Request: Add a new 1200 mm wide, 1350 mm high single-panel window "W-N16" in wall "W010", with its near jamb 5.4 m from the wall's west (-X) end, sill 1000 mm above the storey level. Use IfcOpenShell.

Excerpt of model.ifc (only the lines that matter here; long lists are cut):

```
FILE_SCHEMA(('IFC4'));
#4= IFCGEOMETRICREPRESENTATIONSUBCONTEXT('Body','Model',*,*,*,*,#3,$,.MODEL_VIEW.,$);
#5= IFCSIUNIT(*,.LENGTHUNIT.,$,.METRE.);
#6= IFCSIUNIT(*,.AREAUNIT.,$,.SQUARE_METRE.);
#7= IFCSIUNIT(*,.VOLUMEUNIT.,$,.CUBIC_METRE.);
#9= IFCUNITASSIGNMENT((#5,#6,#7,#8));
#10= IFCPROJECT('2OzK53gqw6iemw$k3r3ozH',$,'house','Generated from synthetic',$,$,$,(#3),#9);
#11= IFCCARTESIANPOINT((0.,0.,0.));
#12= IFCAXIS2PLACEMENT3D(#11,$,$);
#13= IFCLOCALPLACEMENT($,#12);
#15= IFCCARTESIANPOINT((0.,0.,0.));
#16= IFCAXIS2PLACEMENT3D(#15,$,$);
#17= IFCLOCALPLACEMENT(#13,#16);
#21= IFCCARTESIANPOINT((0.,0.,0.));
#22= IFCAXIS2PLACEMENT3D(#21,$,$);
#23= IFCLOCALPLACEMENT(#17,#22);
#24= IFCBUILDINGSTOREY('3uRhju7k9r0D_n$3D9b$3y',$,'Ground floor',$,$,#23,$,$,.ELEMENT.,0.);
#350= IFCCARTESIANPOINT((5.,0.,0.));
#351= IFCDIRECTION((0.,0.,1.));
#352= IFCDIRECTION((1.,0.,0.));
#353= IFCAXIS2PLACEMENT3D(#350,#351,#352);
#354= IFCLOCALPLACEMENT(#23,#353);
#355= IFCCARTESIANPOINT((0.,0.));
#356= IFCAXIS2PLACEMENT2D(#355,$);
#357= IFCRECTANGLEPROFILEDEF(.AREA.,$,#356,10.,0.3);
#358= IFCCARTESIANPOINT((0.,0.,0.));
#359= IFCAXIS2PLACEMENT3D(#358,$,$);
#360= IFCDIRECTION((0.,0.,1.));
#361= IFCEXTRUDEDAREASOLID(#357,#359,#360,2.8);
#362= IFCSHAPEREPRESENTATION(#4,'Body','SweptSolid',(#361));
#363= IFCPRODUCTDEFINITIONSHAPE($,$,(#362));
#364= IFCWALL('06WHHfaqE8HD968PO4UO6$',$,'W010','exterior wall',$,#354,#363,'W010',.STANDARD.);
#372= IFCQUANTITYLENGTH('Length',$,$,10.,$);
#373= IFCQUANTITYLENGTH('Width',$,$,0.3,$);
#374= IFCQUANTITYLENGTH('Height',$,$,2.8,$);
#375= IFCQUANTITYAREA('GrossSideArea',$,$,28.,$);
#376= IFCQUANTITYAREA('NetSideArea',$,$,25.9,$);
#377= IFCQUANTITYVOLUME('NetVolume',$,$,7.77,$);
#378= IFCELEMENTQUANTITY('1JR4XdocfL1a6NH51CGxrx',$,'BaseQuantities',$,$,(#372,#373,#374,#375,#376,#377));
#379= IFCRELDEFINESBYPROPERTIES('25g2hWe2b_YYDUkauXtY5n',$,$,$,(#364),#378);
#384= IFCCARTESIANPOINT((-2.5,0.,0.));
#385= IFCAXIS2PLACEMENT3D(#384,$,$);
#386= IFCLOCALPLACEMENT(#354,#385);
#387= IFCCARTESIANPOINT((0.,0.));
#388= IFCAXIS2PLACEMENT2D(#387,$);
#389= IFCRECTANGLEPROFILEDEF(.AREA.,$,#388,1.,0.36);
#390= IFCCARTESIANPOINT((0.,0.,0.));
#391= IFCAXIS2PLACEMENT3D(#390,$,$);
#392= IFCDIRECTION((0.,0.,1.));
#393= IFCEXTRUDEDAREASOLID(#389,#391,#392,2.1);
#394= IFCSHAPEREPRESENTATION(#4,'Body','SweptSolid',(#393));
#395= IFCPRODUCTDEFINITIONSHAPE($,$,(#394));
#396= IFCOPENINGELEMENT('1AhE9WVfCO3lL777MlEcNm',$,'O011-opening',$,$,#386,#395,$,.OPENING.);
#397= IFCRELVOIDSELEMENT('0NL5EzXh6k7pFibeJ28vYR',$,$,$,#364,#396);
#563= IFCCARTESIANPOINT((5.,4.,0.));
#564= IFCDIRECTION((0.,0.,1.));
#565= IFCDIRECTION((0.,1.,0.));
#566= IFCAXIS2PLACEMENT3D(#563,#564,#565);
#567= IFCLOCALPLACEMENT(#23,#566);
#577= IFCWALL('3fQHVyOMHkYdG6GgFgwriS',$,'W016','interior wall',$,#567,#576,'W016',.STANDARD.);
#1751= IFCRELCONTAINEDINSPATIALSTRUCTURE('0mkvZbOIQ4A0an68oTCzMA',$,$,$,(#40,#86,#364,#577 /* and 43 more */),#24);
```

```python
import numpy as np
import ifcopenshell
import ifcopenshell.api.feature
import ifcopenshell.api.geometry
import ifcopenshell.api.pset
import ifcopenshell.api.root
import ifcopenshell.api.spatial
import ifcopenshell.geom
import ifcopenshell.util.element
import ifcopenshell.util.placement
import ifcopenshell.util.representation
import ifcopenshell.util.shape
import ifcopenshell.util.unit

model = ifcopenshell.open("model.ifc")
unit_scale = ifcopenshell.util.unit.calculate_unit_scale(model)
area_scale = ifcopenshell.util.unit.calculate_unit_scale(model, "AREAUNIT")
volume_scale = ifcopenshell.util.unit.calculate_unit_scale(model, "VOLUMEUNIT")
settings = ifcopenshell.geom.settings()


def volume(element):
    """Net volume in cubic metres, openings subtracted."""
    shape = ifcopenshell.geom.create_shape(settings, element)
    return ifcopenshell.util.shape.get_volume(shape.geometry)


wall = model.by_guid("06WHHfaqE8HD968PO4UO6$")
storey = ifcopenshell.util.element.get_container(wall, ifc_class="IfcBuildingStorey")
context = ifcopenshell.util.representation.get_context(model, "Model", "Body", "MODEL_VIEW")
before = volume(wall)

width, height, from_end, sill = 1.2, 1.35, 5.4, 1  # metres

# The wall runs along its own X axis, and the end named is its -X end.
wall_shape = ifcopenshell.geom.create_shape(settings, wall)
x, y, z = ifcopenshell.util.shape.get_vertices(wall_shape.geometry).T
start = x.min() + from_end
face, thickness = float(y.min()), float(y.max() - y.min())
wall_matrix = ifcopenshell.util.placement.get_local_placement(wall.ObjectPlacement)
level = ifcopenshell.util.placement.get_local_placement(storey.ObjectPlacement)[2, 3]


def in_wall(x, y):
    """Placement at x, y metres in the wall's axes, at sill height."""
    matrix = wall_matrix.copy()
    matrix[:, 3] = wall_matrix @ np.array([x / unit_scale, y / unit_scale, 0.0, 1.0])
    matrix[2, 3] = level + sill / unit_scale
    return matrix


# Opening: a box that overshoots both wall faces by 50 mm.
opening = ifcopenshell.api.root.create_entity(model, ifc_class="IfcOpeningElement", predefined_type="OPENING")
box = ifcopenshell.api.geometry.add_wall_representation(
    model, context=context, length=width, height=height, thickness=thickness + 0.1
)
ifcopenshell.api.geometry.assign_representation(model, product=opening, representation=box)
ifcopenshell.api.geometry.edit_object_placement(model, product=opening, matrix=in_wall(start, face - 0.05), is_si=False)
ifcopenshell.api.feature.add_feature(model, feature=opening, element=wall)

window = ifcopenshell.api.root.create_entity(model, ifc_class="IfcWindow", name="W-N16", predefined_type="WINDOW")
window.OverallWidth, window.OverallHeight = width / unit_scale, height / unit_scale
window.PartitioningType = "SINGLE_PANEL"
body = ifcopenshell.api.geometry.add_window_representation(
    model,
    context=context,
    overall_width=window.OverallWidth,
    overall_height=window.OverallHeight,
    partition_type="SINGLE_PANEL",
)
ifcopenshell.api.geometry.assign_representation(model, product=window, representation=body)
ifcopenshell.api.spatial.assign_container(model, products=[window], relating_structure=storey)
ifcopenshell.api.feature.add_filling(model, opening=opening, element=window)

# Centre the window in the wall's thickness.
ifcopenshell.api.geometry.edit_object_placement(model, product=window, matrix=in_wall(start, face), is_si=False)
window_shape = ifcopenshell.geom.create_shape(settings, window)
depth = ifcopenshell.util.shape.get_vertices(window_shape.geometry)[:, 1]
offset = face + thickness / 2 - (depth.min() + depth.max()) / 2
ifcopenshell.api.geometry.edit_object_placement(model, product=window, matrix=in_wall(start, offset), is_si=False)

after = volume(wall)

# Update the wall's stored quantities.
qto = model.by_id(ifcopenshell.util.element.get_pset(wall, "BaseQuantities", should_inherit=False)["id"])
ifcopenshell.api.pset.edit_qto(model, qto=qto, properties={
    "NetSideArea": after / thickness / area_scale,
    "NetVolume": after / volume_scale,
})

print(f"wall volume {before:.3f} -> {after:.3f} m3")

model.write("model_v2.ifc")
```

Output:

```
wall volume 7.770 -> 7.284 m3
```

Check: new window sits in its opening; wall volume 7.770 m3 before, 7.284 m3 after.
